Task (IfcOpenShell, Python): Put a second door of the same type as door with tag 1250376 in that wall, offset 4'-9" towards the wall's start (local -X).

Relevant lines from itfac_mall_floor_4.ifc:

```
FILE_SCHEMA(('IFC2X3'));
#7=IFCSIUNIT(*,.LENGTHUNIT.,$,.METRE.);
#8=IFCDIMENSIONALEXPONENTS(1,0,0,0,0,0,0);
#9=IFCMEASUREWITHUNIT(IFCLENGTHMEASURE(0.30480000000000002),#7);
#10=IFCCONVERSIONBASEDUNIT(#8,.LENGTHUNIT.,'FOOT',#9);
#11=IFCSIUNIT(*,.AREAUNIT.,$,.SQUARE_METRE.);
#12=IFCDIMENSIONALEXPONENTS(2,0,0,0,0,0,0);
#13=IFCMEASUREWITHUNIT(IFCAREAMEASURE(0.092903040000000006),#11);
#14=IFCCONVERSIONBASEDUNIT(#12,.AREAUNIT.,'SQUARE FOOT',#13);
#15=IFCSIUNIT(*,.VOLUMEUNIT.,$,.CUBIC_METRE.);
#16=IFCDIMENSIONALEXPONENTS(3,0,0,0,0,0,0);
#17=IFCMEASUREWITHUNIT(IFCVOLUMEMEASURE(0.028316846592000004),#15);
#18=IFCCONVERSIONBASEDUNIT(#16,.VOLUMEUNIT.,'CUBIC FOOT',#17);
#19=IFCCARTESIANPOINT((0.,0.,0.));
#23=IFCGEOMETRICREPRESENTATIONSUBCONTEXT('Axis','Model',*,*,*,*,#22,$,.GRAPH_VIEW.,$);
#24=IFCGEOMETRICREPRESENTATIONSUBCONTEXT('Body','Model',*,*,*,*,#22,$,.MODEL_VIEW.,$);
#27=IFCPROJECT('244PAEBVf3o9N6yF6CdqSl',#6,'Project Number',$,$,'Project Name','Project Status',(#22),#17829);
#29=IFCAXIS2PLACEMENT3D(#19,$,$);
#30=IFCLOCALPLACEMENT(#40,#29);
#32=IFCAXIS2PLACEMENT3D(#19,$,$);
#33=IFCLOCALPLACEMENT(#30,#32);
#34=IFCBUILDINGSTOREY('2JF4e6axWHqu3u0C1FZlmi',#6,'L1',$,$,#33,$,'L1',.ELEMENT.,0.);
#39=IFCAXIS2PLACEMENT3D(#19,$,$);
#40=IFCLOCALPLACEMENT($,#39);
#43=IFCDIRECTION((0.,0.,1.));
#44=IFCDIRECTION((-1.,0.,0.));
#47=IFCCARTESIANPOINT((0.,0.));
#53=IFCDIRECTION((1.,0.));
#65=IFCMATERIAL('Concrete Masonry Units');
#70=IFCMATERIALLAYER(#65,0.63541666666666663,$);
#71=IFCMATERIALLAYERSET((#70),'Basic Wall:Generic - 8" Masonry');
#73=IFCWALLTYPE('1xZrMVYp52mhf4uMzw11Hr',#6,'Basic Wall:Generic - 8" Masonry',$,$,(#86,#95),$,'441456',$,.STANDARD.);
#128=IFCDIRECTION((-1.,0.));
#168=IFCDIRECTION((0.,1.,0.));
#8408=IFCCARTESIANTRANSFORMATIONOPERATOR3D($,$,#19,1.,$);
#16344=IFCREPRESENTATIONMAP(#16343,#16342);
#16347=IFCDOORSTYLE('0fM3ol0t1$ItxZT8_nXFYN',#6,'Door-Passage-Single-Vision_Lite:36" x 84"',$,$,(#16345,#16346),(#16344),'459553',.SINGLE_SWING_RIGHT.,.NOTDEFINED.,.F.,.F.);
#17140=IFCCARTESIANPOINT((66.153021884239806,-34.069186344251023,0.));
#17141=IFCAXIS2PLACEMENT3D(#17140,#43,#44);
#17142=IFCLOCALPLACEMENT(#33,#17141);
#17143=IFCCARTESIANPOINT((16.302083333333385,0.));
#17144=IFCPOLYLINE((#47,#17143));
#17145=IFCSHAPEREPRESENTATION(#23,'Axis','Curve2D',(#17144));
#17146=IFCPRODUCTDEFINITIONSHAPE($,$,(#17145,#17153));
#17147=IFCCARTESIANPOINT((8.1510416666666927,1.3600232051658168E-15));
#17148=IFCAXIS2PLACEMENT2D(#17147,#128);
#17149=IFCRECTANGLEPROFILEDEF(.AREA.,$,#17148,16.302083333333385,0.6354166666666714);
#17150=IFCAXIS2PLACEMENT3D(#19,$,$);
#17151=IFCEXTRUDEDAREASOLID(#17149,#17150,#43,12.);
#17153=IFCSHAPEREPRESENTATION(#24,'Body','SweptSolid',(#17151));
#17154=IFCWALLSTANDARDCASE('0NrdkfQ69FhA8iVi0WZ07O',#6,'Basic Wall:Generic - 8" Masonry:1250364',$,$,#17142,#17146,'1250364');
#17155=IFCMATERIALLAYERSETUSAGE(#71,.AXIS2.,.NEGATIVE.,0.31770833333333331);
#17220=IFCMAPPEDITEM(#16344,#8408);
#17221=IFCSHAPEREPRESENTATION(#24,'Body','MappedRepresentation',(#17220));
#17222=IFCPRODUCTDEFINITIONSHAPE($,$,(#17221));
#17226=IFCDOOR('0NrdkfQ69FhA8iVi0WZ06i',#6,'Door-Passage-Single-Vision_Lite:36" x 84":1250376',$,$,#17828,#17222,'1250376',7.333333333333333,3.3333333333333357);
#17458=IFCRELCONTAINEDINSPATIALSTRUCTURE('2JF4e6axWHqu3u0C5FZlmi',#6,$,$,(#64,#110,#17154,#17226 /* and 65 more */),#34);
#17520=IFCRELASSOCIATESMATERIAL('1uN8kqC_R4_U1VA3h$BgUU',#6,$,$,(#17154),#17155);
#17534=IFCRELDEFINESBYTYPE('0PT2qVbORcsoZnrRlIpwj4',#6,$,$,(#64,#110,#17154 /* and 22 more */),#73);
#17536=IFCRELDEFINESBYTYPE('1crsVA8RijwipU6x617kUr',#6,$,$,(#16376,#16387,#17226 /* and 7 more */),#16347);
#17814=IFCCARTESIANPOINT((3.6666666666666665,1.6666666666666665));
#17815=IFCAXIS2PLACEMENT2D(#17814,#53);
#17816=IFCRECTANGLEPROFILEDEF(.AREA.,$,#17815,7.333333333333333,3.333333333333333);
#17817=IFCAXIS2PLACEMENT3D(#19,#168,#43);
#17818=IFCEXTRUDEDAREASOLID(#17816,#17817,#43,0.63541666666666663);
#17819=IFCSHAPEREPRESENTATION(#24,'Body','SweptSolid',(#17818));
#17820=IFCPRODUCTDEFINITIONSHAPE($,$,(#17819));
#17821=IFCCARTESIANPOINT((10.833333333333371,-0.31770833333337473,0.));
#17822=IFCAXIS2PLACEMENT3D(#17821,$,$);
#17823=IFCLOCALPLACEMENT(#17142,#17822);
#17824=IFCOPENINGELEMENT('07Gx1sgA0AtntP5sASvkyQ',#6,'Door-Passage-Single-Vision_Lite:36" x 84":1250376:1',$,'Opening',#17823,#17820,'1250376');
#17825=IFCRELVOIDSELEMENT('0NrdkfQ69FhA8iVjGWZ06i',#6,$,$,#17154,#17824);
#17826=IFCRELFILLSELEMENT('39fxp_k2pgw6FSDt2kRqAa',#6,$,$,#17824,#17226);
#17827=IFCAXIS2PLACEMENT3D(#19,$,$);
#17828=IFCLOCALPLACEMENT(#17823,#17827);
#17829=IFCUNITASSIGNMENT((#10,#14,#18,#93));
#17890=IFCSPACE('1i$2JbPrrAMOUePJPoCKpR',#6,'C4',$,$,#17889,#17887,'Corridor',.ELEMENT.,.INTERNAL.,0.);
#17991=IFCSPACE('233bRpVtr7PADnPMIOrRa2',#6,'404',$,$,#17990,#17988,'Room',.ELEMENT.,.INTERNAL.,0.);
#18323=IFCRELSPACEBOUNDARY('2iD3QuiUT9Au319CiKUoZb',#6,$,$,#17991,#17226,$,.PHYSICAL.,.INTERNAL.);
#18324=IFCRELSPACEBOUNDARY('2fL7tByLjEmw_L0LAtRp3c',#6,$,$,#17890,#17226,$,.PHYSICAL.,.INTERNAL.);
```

```python
import ifcopenshell
import ifcopenshell.api.feature
import ifcopenshell.api.geometry
import ifcopenshell.api.root
import ifcopenshell.geom
import ifcopenshell.util.element
import ifcopenshell.util.placement
import ifcopenshell.util.shape
import ifcopenshell.util.unit

model = ifcopenshell.open("itfac_mall_floor_4.ifc")
unit_scale = ifcopenshell.util.unit.calculate_unit_scale(model)
settings = ifcopenshell.geom.settings()


def volume(element):
    """Net volume in cubic metres, openings subtracted."""
    shape = ifcopenshell.geom.create_shape(settings, element)
    return ifcopenshell.util.shape.get_volume(shape.geometry)


def reuse_history(source, copy):
    """copy_class also copies each property set's owner history, people and application; keep the originals."""
    for rel in copy.IsDefinedBy:
        if rel.is_a("IfcRelDefinesByProperties") and (history := rel.RelatingPropertyDefinition.OwnerHistory):
            rel.RelatingPropertyDefinition.OwnerHistory = source.OwnerHistory
            ifcopenshell.util.element.remove_deep2(model, history)


door = model.by_guid("0NrdkfQ69FhA8iVi0WZ06i")
opening = door.FillsVoids[0].RelatingOpeningElement
wall = opening.VoidsElements[0].RelatingBuildingElement
before = volume(wall)
shift = ifcopenshell.util.placement.get_local_placement(wall.ObjectPlacement)[:3, 0] * -57 * 0.0254 / unit_scale

# copy_class copies the void relationship, type, container and properties, but no geometry.
new_opening = ifcopenshell.api.root.copy_class(model, product=opening)
new_opening.Representation = ifcopenshell.util.element.copy_deep(
    model, opening.Representation, exclude=["IfcGeometricRepresentationContext", "IfcRepresentationMap"]
)
new_opening.Name = 'Door-Passage-Single-Vision_Lite:36" x 84"'
new_opening.Tag = None
new_door = ifcopenshell.api.root.copy_class(model, product=door)
new_door.Representation = ifcopenshell.util.element.copy_deep(
    model, door.Representation, exclude=["IfcGeometricRepresentationContext", "IfcRepresentationMap"]
)
new_door.Name = 'Door-Passage-Single-Vision_Lite:36" x 84"'
new_door.Tag = None
reuse_history(door, new_door)
fills = ifcopenshell.api.feature.add_filling(model, opening=new_opening, element=new_door)
fills.OwnerHistory = new_door.OwnerHistory  # required in IFC2X3

for old, new in ((opening, new_opening), (door, new_door)):
    matrix = ifcopenshell.util.placement.get_local_placement(old.ObjectPlacement)
    matrix[:3, 3] += shift
    ifcopenshell.api.geometry.edit_object_placement(model, product=new, matrix=matrix, is_si=False)

after = volume(wall)

print(f"wall volume {before:.3f} -> {after:.3f} m3")

model.write("itfac_mall_floor_4_v2.ifc")
```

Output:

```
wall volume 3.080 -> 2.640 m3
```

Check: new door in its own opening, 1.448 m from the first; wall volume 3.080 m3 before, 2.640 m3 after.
